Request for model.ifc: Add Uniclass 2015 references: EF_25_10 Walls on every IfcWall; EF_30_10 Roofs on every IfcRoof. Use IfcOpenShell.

First a look at what the model holds.

```python
import ifcopenshell

model = ifcopenshell.open("model.ifc")
print(model.schema)
print("classifications:", [c.Name for c in model.by_type("IfcClassification")])
for ifc_class in ("IfcDoor", "IfcRoof", "IfcStair", "IfcWall", "IfcWindow"):
    print(ifc_class, len(model.by_type(ifc_class)))
```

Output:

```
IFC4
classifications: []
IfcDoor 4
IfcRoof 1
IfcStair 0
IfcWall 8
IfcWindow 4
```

```python
import ifcopenshell
import ifcopenshell.api.classification

model = ifcopenshell.open("model.ifc")

system = ifcopenshell.api.classification.add_classification(model, classification="Uniclass 2015")

codes = {
    "IfcWall": ("EF_25_10", "Walls"),
    "IfcRoof": ("EF_30_10", "Roofs"),
}
for ifc_class, (code, name) in codes.items():
    products = model.by_type(ifc_class)
    ifcopenshell.api.classification.add_reference(
        model, products=products, classification=system, identification=code, name=name
    )
    print(code, len(products))

model.write("model_rev.ifc")
```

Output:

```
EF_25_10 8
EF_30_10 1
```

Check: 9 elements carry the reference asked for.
